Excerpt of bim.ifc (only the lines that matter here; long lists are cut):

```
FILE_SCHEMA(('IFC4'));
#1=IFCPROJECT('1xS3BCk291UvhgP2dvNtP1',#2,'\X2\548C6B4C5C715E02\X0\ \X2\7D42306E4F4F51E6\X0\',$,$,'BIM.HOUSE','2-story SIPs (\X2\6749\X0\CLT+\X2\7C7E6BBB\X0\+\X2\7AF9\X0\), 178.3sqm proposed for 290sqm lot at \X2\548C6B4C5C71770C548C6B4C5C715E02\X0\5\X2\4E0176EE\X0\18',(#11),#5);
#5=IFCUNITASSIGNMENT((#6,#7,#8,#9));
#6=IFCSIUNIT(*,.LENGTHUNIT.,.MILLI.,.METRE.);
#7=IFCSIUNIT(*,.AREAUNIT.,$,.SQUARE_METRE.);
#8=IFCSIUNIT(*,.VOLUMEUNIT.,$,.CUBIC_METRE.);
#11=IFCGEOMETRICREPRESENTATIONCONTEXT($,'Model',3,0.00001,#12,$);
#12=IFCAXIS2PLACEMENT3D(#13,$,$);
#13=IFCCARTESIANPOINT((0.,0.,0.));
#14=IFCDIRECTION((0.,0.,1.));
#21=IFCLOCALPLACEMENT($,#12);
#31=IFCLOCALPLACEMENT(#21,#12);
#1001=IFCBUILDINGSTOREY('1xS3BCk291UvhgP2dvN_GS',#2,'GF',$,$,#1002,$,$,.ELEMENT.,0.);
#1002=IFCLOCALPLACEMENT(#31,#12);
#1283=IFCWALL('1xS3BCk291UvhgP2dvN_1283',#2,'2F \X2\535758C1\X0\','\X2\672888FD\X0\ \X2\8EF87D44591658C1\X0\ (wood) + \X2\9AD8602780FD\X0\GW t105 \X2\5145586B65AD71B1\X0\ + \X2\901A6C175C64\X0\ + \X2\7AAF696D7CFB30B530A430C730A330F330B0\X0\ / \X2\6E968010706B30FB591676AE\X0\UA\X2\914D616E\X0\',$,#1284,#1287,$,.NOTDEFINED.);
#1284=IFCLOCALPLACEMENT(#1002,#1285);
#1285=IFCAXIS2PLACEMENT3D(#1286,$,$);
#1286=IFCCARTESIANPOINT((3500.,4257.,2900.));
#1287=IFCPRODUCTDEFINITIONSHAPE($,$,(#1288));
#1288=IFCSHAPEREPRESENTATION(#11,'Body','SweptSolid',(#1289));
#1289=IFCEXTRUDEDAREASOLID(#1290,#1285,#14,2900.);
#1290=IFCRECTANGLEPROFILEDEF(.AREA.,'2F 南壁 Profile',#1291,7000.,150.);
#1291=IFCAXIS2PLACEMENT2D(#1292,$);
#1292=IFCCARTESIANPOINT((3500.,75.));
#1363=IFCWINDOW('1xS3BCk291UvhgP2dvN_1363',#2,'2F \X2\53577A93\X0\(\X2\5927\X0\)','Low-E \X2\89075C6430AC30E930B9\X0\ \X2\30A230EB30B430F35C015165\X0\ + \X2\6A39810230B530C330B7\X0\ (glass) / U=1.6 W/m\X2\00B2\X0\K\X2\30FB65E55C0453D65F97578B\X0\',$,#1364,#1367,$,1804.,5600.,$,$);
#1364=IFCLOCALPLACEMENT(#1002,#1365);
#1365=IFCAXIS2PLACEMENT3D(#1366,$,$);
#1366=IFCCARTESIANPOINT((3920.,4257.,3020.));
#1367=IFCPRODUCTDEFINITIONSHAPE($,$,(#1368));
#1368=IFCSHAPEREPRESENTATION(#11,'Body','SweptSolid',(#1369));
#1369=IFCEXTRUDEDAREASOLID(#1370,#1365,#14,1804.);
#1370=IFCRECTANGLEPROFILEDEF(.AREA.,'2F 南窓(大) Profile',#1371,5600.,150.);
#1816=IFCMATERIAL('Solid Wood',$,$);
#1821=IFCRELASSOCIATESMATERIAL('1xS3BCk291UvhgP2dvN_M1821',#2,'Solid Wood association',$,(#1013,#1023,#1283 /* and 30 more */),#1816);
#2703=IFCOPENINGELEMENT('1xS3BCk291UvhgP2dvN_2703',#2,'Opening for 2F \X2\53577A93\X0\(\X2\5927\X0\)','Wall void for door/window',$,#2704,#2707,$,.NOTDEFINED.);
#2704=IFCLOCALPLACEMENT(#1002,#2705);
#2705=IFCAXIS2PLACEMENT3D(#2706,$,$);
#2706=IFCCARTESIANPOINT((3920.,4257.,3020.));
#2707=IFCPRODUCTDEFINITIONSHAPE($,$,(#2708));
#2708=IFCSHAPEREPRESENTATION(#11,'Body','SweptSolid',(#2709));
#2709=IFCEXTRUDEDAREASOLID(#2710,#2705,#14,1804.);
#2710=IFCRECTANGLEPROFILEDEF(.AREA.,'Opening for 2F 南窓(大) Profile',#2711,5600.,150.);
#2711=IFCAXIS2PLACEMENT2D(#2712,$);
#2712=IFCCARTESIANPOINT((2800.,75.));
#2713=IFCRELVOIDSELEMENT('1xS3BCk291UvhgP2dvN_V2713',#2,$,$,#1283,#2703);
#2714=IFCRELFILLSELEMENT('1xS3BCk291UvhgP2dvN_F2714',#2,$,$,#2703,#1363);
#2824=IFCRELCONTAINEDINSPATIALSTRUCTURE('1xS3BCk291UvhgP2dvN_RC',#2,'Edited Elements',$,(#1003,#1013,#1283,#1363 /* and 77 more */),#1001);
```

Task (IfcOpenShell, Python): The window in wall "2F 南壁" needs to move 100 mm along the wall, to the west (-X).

```python
import ifcopenshell
import ifcopenshell.api.geometry
import ifcopenshell.util.placement

model = ifcopenshell.open("bim.ifc")

window = model.by_id(1363)
opening = window.FillsVoids[0].RelatingOpeningElement
wall = opening.VoidsElements[0].RelatingBuildingElement

wall_matrix = ifcopenshell.util.placement.get_local_placement(wall.ObjectPlacement)
shift = wall_matrix[:3, 0] * -100.0
before = ifcopenshell.util.placement.get_local_placement(window.ObjectPlacement)[:3, 3].copy()

# The window is not placed relative to its opening, so move both.
for product in (opening, window):
    matrix = ifcopenshell.util.placement.get_local_placement(product.ObjectPlacement)
    matrix[:3, 3] += shift
    ifcopenshell.api.geometry.edit_object_placement(model, product=product, matrix=matrix, is_si=False)

after = ifcopenshell.util.placement.get_local_placement(window.ObjectPlacement)[:3, 3]
print("window moved by", (after - before).round(3) + 0.0)

model.write("bim-out.ifc")
```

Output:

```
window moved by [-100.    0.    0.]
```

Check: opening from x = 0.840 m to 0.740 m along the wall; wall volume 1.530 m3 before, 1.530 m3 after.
